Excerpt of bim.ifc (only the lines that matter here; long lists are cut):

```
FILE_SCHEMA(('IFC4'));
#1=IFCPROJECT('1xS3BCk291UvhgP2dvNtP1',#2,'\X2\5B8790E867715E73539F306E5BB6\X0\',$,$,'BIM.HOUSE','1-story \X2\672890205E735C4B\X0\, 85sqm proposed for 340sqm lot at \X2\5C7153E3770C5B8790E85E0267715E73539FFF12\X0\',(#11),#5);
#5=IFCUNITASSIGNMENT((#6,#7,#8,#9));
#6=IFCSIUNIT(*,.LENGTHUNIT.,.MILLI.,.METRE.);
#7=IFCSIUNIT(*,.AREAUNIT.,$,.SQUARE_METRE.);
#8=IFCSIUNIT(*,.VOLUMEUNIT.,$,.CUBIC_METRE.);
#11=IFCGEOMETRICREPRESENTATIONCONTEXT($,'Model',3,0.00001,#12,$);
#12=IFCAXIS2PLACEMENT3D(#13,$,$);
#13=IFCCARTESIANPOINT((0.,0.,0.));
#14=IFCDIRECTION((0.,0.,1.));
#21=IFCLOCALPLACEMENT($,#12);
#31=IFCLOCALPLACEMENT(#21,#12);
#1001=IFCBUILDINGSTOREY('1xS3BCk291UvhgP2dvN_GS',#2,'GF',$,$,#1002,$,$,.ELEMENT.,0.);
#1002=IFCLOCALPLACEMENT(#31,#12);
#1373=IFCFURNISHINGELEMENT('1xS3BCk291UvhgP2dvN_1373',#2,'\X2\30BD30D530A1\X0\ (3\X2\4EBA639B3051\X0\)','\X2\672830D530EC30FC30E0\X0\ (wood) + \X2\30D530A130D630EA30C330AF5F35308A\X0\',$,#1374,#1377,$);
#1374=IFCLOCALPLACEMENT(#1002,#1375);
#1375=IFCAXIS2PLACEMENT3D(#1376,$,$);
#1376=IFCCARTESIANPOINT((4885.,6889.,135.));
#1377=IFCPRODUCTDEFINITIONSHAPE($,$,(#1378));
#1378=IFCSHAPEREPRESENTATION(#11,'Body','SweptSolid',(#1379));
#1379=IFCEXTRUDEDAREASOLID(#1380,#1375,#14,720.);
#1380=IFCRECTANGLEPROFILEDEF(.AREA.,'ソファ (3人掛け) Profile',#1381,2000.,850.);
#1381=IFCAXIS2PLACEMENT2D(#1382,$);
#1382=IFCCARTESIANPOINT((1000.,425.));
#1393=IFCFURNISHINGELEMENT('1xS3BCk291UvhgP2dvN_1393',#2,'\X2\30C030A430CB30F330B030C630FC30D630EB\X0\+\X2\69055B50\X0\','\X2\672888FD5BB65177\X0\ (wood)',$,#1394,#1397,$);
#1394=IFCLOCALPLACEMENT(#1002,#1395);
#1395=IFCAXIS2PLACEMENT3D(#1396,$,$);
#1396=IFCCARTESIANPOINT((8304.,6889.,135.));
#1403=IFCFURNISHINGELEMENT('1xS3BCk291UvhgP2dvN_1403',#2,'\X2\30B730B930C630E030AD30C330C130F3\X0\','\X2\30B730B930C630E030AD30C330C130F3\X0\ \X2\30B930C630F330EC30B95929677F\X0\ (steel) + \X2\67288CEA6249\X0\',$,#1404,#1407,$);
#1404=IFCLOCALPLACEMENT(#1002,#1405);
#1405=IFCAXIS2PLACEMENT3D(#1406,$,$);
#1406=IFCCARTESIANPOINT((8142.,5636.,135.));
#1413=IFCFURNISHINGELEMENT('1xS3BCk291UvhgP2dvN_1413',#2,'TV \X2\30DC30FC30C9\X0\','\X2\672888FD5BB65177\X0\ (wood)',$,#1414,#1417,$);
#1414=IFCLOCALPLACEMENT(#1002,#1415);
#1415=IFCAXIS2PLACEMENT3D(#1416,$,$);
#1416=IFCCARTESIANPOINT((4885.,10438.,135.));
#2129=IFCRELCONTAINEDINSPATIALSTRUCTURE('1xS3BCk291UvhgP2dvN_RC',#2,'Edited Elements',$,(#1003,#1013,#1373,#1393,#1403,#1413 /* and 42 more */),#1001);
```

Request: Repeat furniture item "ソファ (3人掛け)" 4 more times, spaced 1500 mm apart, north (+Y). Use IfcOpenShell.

```python
import numpy as np
import ifcopenshell
import ifcopenshell.api.geometry
import ifcopenshell.api.root
import ifcopenshell.util.element
import ifcopenshell.util.placement

model = ifcopenshell.open("bim.ifc")


def reuse_history(source, copy):
    """copy_class also copies each property set's owner history, people and application; keep the originals."""
    for rel in copy.IsDefinedBy:
        if rel.is_a("IfcRelDefinesByProperties") and (history := rel.RelatingPropertyDefinition.OwnerHistory):
            rel.RelatingPropertyDefinition.OwnerHistory = source.OwnerHistory
            ifcopenshell.util.element.remove_deep2(model, history)


source = model.by_id(1373)
base = ifcopenshell.util.placement.get_local_placement(source.ObjectPlacement)
step = np.array([0.0, 1.0, 0.0]) * 1500.0

for i in range(1, 5):
    copy = ifcopenshell.api.root.copy_class(model, product=source)
    copy.Representation = ifcopenshell.util.element.copy_deep(
        model, source.Representation, exclude=["IfcGeometricRepresentationContext", "IfcRepresentationMap"]
    )
    reuse_history(source, copy)
    matrix = base.copy()
    matrix[:3, 3] += i * step
    print("added at", matrix[:3, 3].round(3) + 0.0)
    ifcopenshell.api.geometry.edit_object_placement(model, product=copy, matrix=matrix, is_si=False)

model.write("bim_rev.ifc")
```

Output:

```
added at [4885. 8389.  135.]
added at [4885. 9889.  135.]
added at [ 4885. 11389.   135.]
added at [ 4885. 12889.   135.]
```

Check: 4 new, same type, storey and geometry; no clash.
